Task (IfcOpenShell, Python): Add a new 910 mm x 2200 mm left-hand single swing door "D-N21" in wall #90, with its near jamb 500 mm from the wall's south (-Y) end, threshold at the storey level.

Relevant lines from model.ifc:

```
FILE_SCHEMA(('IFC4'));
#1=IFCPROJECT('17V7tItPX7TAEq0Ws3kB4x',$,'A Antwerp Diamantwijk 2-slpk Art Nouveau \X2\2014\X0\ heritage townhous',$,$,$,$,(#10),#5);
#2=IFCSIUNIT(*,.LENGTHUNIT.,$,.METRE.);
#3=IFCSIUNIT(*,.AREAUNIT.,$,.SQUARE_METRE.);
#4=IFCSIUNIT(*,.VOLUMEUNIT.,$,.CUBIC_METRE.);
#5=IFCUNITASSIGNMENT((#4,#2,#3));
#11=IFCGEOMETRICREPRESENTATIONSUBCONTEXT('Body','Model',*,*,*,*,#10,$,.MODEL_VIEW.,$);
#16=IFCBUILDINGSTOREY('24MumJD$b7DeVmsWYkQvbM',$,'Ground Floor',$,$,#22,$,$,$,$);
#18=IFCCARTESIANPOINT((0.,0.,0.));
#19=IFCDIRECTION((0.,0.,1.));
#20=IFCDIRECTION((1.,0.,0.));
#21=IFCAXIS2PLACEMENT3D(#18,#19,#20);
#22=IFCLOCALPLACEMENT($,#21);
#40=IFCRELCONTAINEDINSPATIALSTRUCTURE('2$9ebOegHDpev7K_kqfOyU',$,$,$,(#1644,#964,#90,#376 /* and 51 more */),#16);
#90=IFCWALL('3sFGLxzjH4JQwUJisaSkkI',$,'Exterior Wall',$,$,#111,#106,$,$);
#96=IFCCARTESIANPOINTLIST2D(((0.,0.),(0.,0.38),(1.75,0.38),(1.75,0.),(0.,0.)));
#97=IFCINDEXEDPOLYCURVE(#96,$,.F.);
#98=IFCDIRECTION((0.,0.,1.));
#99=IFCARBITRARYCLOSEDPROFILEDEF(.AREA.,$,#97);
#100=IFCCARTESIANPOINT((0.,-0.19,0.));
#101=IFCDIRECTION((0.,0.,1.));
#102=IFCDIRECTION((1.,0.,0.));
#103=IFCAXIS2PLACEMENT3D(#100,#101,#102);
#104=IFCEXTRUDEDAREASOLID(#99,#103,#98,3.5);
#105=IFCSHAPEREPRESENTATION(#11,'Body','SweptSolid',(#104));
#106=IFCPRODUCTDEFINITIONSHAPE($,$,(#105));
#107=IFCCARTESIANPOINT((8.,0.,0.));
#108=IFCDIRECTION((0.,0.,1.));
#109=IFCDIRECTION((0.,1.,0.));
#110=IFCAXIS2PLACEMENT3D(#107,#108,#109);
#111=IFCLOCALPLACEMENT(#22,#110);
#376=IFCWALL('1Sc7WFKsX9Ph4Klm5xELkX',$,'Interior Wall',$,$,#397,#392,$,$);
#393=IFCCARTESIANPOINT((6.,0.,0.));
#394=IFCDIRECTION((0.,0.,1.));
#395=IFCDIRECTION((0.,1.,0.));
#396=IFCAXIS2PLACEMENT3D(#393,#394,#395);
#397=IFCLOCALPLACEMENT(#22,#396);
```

```python
import numpy as np
import ifcopenshell
import ifcopenshell.api.feature
import ifcopenshell.api.geometry
import ifcopenshell.api.root
import ifcopenshell.api.spatial
import ifcopenshell.geom
import ifcopenshell.util.element
import ifcopenshell.util.placement
import ifcopenshell.util.representation
import ifcopenshell.util.shape
import ifcopenshell.util.unit

model = ifcopenshell.open("model.ifc")
unit_scale = ifcopenshell.util.unit.calculate_unit_scale(model)
settings = ifcopenshell.geom.settings()


def volume(element):
    """Net volume in cubic metres, openings subtracted."""
    shape = ifcopenshell.geom.create_shape(settings, element)
    return ifcopenshell.util.shape.get_volume(shape.geometry)


wall = model.by_id(90)
storey = ifcopenshell.util.element.get_container(wall, ifc_class="IfcBuildingStorey")
context = ifcopenshell.util.representation.get_context(model, "Model", "Body", "MODEL_VIEW")
before = volume(wall)

width, height, from_end, sill = 0.91, 2.2, 0.5, 0.0  # metres

# The wall runs along its own X axis, and the end named is its -X end.
wall_shape = ifcopenshell.geom.create_shape(settings, wall)
x, y, z = ifcopenshell.util.shape.get_vertices(wall_shape.geometry).T
start = x.min() + from_end
face, thickness = float(y.min()), float(y.max() - y.min())
wall_matrix = ifcopenshell.util.placement.get_local_placement(wall.ObjectPlacement)
level = ifcopenshell.util.placement.get_local_placement(storey.ObjectPlacement)[2, 3]


def in_wall(x, y):
    """Placement at x, y metres in the wall's axes, at sill height."""
    matrix = wall_matrix.copy()
    matrix[:, 3] = wall_matrix @ np.array([x / unit_scale, y / unit_scale, 0.0, 1.0])
    matrix[2, 3] = level + sill / unit_scale
    return matrix


# Opening: a box that overshoots both wall faces by 50 mm.
opening = ifcopenshell.api.root.create_entity(model, ifc_class="IfcOpeningElement", predefined_type="OPENING")
box = ifcopenshell.api.geometry.add_wall_representation(
    model, context=context, length=width, height=height, thickness=thickness + 0.1
)
ifcopenshell.api.geometry.assign_representation(model, product=opening, representation=box)
ifcopenshell.api.geometry.edit_object_placement(model, product=opening, matrix=in_wall(start, face - 0.05), is_si=False)
ifcopenshell.api.feature.add_feature(model, feature=opening, element=wall)

door = ifcopenshell.api.root.create_entity(model, ifc_class="IfcDoor", name="D-N21", predefined_type="DOOR")
door.OverallWidth, door.OverallHeight = width / unit_scale, height / unit_scale
door.OperationType = "SINGLE_SWING_LEFT"
body = ifcopenshell.api.geometry.add_door_representation(
    model,
    context=context,
    overall_width=door.OverallWidth,
    overall_height=door.OverallHeight,
    operation_type="SINGLE_SWING_LEFT",
    lining_properties={"LiningDepth": thickness / unit_scale, "ThresholdDepth": thickness / unit_scale},
)
ifcopenshell.api.geometry.assign_representation(model, product=door, representation=body)
ifcopenshell.api.spatial.assign_container(model, products=[door], relating_structure=storey)
ifcopenshell.api.feature.add_filling(model, opening=opening, element=door)

# The lining spans the wall, so the door starts at the wall face.
ifcopenshell.api.geometry.edit_object_placement(model, product=door, matrix=in_wall(start, face), is_si=False)

after = volume(wall)

print(f"wall volume {before:.3f} -> {after:.3f} m3")

model.write("model_edited.ifc")
```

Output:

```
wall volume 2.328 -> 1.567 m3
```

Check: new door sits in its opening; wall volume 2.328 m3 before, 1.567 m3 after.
